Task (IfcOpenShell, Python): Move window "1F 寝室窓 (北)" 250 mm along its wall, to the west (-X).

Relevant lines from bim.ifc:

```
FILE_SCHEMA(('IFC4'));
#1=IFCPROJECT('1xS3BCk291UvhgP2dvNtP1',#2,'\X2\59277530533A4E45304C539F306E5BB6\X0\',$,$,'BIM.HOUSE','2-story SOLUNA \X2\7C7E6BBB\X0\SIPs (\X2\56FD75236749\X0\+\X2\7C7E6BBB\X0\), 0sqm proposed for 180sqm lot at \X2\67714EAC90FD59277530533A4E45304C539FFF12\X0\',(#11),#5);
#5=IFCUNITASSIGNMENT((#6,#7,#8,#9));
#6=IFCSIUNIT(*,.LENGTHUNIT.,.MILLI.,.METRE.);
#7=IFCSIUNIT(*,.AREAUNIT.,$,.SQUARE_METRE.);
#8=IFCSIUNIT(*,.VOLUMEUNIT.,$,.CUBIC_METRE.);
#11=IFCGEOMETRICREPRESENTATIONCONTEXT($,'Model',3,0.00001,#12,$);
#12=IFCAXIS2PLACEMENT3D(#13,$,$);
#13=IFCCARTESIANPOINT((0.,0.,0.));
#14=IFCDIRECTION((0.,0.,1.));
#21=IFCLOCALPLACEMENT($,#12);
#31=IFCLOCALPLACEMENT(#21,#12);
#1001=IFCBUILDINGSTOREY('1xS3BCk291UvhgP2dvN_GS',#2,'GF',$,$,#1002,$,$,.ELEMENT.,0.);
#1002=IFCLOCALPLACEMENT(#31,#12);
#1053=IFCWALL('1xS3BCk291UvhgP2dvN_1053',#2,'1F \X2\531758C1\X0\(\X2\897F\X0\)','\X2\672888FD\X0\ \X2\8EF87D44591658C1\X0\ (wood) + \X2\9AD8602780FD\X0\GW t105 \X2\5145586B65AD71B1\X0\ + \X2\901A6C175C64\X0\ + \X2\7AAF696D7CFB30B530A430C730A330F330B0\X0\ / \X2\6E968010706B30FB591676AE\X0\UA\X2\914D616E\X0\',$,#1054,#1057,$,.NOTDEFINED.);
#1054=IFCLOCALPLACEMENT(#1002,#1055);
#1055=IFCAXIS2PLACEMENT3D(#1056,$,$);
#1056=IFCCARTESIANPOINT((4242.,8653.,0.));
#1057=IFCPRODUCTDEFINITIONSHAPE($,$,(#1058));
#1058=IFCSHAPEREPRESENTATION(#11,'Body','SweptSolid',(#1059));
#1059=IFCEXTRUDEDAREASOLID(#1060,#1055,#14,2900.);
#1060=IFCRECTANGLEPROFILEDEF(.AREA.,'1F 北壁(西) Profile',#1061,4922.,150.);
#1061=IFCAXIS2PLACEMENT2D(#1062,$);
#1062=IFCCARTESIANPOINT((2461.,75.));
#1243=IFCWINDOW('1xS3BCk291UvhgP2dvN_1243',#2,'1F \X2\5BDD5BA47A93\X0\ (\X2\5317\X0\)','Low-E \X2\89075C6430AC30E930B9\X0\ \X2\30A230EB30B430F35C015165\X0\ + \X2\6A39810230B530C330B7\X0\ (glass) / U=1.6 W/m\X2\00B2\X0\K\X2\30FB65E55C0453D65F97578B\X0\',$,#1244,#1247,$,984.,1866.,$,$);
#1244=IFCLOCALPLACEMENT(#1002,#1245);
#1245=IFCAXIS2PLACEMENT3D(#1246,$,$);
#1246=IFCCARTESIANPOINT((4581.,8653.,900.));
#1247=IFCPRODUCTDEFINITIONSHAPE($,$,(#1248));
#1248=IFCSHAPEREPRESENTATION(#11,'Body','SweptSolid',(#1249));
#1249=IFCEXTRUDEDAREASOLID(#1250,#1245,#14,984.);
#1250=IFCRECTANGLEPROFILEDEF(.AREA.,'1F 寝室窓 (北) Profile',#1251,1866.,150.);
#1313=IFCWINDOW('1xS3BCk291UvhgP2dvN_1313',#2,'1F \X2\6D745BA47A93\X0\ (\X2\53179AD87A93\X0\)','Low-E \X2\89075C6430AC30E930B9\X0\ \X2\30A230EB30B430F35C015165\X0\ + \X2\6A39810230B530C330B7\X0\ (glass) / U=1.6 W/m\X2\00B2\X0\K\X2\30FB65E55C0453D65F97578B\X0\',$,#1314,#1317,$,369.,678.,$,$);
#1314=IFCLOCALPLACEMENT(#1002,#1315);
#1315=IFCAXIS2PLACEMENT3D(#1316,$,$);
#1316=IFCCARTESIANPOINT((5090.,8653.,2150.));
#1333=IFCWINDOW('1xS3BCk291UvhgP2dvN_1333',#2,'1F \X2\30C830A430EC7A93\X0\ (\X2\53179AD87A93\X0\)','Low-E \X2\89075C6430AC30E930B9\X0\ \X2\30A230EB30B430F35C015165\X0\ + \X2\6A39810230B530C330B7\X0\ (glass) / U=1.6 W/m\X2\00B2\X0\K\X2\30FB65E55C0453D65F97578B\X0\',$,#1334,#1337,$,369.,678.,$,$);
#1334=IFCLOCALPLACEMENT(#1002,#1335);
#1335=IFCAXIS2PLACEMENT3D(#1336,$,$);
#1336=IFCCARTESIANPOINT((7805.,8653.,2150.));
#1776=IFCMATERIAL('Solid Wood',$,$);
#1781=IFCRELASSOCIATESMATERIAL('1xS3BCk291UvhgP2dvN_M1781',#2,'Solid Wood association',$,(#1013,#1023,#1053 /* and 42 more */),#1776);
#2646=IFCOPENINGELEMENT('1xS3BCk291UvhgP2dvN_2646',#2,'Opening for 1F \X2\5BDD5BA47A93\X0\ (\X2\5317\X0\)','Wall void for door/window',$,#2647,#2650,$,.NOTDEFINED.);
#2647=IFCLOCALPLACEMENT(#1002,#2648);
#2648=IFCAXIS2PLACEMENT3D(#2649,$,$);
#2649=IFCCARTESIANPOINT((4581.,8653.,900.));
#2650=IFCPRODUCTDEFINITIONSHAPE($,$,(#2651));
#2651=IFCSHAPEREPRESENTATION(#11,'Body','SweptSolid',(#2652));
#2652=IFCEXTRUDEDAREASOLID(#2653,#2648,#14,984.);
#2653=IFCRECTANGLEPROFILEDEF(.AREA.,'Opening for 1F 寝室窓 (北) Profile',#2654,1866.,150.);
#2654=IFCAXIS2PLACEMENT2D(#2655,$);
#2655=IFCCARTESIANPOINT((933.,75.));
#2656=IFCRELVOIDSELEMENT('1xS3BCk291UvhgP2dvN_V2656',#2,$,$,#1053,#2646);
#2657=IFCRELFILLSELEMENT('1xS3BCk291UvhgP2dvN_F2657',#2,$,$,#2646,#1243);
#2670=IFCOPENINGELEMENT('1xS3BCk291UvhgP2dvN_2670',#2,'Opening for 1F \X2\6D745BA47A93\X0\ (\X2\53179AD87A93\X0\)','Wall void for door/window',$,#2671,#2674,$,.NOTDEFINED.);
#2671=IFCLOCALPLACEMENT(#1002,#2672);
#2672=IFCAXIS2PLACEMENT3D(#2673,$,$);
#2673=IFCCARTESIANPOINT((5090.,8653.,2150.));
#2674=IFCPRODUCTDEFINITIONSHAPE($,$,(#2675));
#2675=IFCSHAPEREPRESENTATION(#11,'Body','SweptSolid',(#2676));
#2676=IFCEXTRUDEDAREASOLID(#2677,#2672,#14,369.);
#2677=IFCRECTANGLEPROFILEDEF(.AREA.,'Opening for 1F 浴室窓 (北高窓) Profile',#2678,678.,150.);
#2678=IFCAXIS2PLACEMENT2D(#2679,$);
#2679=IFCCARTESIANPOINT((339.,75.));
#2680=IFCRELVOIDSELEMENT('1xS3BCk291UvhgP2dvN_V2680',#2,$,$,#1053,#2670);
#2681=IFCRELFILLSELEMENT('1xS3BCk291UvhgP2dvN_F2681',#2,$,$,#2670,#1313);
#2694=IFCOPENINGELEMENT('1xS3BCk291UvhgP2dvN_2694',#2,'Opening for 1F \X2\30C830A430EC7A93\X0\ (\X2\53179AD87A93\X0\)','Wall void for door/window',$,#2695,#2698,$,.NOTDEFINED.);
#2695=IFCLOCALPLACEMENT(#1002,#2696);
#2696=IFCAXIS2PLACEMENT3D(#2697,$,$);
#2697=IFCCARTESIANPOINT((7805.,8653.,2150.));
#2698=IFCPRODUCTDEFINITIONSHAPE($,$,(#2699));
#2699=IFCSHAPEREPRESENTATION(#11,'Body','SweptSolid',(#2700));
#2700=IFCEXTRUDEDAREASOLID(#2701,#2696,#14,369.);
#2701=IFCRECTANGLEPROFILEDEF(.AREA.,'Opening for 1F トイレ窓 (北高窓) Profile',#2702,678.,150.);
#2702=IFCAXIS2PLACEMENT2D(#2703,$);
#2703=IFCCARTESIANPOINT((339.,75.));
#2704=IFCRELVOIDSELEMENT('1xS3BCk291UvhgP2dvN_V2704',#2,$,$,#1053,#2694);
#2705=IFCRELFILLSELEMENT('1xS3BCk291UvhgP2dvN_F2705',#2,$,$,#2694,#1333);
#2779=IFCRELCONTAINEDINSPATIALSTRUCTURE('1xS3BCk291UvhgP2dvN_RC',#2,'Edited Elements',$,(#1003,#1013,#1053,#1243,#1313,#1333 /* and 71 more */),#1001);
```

```python
import ifcopenshell
import ifcopenshell.api.geometry
import ifcopenshell.util.placement
import ifcopenshell.util.unit

model = ifcopenshell.open("bim.ifc")
unit_scale = ifcopenshell.util.unit.calculate_unit_scale(model)

window = model.by_id(1243)
opening = window.FillsVoids[0].RelatingOpeningElement
wall = opening.VoidsElements[0].RelatingBuildingElement

wall_matrix = ifcopenshell.util.placement.get_local_placement(wall.ObjectPlacement)
shift = wall_matrix[:3, 0] * -0.25 / unit_scale
before = ifcopenshell.util.placement.get_local_placement(window.ObjectPlacement)[:3, 3].copy()

# The window is not placed relative to its opening, so move both.
for product in (opening, window):
    matrix = ifcopenshell.util.placement.get_local_placement(product.ObjectPlacement)
    matrix[:3, 3] += shift
    ifcopenshell.api.geometry.edit_object_placement(model, product=product, matrix=matrix, is_si=False)

after = ifcopenshell.util.placement.get_local_placement(window.ObjectPlacement)[:3, 3]
print("window moved by", (after - before).round(3) + 0.0)

model.write("bim-out.ifc")
```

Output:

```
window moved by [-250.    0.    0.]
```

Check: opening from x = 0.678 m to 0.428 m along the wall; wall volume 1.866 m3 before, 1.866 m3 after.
